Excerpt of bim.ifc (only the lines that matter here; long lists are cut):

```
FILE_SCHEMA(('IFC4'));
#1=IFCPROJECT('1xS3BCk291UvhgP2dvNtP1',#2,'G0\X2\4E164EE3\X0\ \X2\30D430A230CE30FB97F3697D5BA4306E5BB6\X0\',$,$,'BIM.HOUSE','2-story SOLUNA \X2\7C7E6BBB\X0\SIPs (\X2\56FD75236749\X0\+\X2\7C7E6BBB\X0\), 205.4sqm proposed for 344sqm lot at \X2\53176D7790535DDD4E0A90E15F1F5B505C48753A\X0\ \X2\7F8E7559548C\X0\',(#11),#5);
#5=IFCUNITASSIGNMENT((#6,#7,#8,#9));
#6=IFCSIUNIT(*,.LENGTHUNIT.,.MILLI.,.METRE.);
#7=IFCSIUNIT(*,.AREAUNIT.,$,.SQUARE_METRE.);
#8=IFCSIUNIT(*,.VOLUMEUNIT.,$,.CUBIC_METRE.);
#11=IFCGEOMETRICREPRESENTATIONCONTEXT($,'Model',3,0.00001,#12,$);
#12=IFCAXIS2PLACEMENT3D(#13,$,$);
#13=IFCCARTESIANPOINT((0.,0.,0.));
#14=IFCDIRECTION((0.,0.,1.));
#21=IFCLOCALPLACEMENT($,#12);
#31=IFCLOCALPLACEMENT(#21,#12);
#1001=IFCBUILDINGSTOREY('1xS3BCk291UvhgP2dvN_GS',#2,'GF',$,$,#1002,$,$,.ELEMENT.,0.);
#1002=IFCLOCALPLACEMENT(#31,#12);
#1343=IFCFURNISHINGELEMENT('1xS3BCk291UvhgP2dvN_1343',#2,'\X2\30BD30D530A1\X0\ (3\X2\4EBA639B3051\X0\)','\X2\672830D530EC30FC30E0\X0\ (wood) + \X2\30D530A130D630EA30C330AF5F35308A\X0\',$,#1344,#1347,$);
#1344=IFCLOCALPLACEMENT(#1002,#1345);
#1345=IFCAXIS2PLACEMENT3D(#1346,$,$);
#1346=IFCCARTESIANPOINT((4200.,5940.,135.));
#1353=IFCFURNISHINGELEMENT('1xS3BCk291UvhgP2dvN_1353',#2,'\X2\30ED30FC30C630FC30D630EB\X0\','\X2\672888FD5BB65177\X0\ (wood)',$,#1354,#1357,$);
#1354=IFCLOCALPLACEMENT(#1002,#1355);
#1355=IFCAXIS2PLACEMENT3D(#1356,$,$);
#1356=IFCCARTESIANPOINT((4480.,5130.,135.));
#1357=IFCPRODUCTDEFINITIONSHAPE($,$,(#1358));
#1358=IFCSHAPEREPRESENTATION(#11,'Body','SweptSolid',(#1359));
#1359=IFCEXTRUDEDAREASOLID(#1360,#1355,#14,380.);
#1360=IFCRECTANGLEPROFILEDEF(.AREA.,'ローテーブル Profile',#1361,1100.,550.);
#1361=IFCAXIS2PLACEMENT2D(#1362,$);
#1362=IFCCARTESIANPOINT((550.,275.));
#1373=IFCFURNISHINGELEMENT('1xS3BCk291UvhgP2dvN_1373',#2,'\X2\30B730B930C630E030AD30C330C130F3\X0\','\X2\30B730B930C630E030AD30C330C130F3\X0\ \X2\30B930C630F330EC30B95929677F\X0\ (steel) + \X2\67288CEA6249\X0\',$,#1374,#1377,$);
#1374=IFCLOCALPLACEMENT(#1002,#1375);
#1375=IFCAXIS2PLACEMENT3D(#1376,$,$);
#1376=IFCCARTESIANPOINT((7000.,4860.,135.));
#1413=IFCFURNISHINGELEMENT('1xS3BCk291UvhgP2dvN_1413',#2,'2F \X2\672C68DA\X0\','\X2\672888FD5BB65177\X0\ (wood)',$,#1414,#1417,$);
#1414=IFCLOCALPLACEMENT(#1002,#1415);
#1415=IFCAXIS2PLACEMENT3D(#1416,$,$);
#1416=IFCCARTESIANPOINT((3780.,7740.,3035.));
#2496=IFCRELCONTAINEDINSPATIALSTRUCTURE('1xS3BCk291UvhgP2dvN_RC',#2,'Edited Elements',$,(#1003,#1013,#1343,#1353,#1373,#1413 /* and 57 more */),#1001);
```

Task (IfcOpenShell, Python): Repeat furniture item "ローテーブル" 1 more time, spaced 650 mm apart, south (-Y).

```python
import numpy as np
import ifcopenshell
import ifcopenshell.api.geometry
import ifcopenshell.api.root
import ifcopenshell.util.element
import ifcopenshell.util.placement
import ifcopenshell.util.unit

model = ifcopenshell.open("bim.ifc")
unit_scale = ifcopenshell.util.unit.calculate_unit_scale(model)


def reuse_history(source, copy):
    """copy_class also copies each property set's owner history, people and application; keep the originals."""
    for rel in copy.IsDefinedBy:
        if rel.is_a("IfcRelDefinesByProperties") and (history := rel.RelatingPropertyDefinition.OwnerHistory):
            rel.RelatingPropertyDefinition.OwnerHistory = source.OwnerHistory
            ifcopenshell.util.element.remove_deep2(model, history)


source = model.by_guid("1xS3BCk291UvhgP2dvN_1353")
base = ifcopenshell.util.placement.get_local_placement(source.ObjectPlacement)
step = np.array([0.0, -1.0, 0.0]) * 0.65 / unit_scale

for i in range(1, 2):
    copy = ifcopenshell.api.root.copy_class(model, product=source)
    copy.Representation = ifcopenshell.util.element.copy_deep(
        model, source.Representation, exclude=["IfcGeometricRepresentationContext", "IfcRepresentationMap"]
    )
    reuse_history(source, copy)
    matrix = base.copy()
    matrix[:3, 3] += i * step
    print("added at", matrix[:3, 3].round(3) + 0.0)
    ifcopenshell.api.geometry.edit_object_placement(model, product=copy, matrix=matrix, is_si=False)

model.write("bim_edited.ifc")
```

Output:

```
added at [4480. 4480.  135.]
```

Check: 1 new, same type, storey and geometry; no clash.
